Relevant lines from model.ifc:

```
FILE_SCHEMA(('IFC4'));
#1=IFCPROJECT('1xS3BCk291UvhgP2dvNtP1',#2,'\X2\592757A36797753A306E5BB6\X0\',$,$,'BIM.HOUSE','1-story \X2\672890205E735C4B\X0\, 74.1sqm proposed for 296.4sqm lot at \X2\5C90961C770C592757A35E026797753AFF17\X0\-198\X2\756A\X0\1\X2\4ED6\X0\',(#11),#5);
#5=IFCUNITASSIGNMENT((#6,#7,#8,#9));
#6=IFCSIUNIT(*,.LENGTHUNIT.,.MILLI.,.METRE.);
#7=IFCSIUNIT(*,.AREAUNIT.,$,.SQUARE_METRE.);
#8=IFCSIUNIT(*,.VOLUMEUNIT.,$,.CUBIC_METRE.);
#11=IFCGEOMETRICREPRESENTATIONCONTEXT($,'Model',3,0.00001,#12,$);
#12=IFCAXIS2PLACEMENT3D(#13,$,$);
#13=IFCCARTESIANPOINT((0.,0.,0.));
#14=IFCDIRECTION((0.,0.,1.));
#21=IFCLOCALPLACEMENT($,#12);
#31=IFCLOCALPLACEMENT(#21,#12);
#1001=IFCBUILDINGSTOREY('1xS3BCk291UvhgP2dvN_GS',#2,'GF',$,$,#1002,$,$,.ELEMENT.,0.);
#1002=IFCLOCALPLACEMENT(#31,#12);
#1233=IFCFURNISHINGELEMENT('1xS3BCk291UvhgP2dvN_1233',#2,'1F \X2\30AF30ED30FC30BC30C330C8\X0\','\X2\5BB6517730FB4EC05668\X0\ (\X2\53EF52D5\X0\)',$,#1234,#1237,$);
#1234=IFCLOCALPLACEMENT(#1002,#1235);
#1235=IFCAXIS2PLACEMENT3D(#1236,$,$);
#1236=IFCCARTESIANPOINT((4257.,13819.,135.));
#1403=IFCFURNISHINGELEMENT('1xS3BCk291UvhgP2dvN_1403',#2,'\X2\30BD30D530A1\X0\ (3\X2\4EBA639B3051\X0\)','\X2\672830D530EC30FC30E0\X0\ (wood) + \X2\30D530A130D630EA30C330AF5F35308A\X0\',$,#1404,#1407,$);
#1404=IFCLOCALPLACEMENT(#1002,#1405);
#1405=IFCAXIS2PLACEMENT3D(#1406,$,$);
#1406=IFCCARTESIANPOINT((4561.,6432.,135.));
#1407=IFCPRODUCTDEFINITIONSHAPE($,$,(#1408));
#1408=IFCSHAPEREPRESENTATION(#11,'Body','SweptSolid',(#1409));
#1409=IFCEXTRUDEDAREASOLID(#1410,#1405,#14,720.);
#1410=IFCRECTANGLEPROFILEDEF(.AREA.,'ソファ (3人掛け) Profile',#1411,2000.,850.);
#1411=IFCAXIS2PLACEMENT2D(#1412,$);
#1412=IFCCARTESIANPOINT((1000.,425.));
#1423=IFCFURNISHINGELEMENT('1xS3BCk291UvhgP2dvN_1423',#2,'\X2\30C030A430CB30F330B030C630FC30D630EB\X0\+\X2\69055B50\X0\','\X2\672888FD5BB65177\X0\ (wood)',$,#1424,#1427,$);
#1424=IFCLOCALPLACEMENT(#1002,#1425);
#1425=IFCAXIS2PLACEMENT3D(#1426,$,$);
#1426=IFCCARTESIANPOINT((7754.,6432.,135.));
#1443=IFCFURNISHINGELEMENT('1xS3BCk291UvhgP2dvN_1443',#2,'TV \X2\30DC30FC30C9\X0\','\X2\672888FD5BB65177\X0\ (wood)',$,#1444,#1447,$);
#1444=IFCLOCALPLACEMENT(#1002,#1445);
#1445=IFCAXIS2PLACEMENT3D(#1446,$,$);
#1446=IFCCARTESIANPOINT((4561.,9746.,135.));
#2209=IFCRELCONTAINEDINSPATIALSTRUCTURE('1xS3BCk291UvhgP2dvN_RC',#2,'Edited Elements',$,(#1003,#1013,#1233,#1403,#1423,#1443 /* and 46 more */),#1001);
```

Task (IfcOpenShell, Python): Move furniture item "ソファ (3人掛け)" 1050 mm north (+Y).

```python
import ifcopenshell
import ifcopenshell.api.geometry
import ifcopenshell.util.placement

model = ifcopenshell.open("model.ifc")

item = model.by_id(1403)
matrix = ifcopenshell.util.placement.get_local_placement(item.ObjectPlacement)
matrix[1, 3] += 1050.0
ifcopenshell.api.geometry.edit_object_placement(model, product=item, matrix=matrix, is_si=False)

print(ifcopenshell.util.placement.get_local_placement(item.ObjectPlacement).round(3) + 0.0)

model.write("model-out.ifc")
```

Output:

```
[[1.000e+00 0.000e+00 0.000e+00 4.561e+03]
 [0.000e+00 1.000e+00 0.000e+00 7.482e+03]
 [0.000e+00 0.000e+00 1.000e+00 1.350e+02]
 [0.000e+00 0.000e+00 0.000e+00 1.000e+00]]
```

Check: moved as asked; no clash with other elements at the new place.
